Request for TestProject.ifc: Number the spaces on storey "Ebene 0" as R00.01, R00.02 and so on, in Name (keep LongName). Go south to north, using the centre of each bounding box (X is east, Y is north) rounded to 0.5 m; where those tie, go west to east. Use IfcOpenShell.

First a look at what the model holds.

```python
import ifcopenshell
import ifcopenshell.util.element
import ifcopenshell.util.placement

model = ifcopenshell.open("TestProject.ifc")
print(model.schema)
storey = next(s for s in model.by_type("IfcBuildingStorey") if s.Name == "Ebene 0")
spaces = [e for e in ifcopenshell.util.element.get_decomposition(storey) if e.is_a("IfcSpace")]
for e in sorted(spaces, key=lambda e: e.id()):
    origin = ifcopenshell.util.placement.get_local_placement(e.ObjectPlacement)[:3, 3]
    print(e.id(), e.Name, e.LongName, origin.round(2) + 0.0, sep=" | ")
```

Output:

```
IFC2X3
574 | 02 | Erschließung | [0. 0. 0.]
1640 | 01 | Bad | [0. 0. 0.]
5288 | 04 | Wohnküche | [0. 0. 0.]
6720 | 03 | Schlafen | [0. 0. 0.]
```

```python
import ifcopenshell
import ifcopenshell.geom
import ifcopenshell.util.element
import ifcopenshell.util.shape

model = ifcopenshell.open("TestProject.ifc")
settings = ifcopenshell.geom.settings()
settings.set("use-world-coords", True)


def centre(element):
    shape = ifcopenshell.geom.create_shape(settings, element)
    return ifcopenshell.util.shape.get_bbox_centroid(shape.geometry)


storey = next(s for s in model.by_type("IfcBuildingStorey") if s.Name == "Ebene 0")
spaces = [e for e in ifcopenshell.util.element.get_decomposition(storey) if e.is_a("IfcSpace")]

# Insertion points can sit at a corner or the storey origin, so sort by the geometry (in metres).
centres = {e: centre(e) for e in spaces}
spaces.sort(key=lambda e: (round(centres[e][1] / 0.5), centres[e][0]))

for i, e in enumerate(spaces, start=1):
    number = f"R00.{i:02d}"
    e.Name = number
    print(e.id(), number)

model.write("TestProject_rev.ifc")
```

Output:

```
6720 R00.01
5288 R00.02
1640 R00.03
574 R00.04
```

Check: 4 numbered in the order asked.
